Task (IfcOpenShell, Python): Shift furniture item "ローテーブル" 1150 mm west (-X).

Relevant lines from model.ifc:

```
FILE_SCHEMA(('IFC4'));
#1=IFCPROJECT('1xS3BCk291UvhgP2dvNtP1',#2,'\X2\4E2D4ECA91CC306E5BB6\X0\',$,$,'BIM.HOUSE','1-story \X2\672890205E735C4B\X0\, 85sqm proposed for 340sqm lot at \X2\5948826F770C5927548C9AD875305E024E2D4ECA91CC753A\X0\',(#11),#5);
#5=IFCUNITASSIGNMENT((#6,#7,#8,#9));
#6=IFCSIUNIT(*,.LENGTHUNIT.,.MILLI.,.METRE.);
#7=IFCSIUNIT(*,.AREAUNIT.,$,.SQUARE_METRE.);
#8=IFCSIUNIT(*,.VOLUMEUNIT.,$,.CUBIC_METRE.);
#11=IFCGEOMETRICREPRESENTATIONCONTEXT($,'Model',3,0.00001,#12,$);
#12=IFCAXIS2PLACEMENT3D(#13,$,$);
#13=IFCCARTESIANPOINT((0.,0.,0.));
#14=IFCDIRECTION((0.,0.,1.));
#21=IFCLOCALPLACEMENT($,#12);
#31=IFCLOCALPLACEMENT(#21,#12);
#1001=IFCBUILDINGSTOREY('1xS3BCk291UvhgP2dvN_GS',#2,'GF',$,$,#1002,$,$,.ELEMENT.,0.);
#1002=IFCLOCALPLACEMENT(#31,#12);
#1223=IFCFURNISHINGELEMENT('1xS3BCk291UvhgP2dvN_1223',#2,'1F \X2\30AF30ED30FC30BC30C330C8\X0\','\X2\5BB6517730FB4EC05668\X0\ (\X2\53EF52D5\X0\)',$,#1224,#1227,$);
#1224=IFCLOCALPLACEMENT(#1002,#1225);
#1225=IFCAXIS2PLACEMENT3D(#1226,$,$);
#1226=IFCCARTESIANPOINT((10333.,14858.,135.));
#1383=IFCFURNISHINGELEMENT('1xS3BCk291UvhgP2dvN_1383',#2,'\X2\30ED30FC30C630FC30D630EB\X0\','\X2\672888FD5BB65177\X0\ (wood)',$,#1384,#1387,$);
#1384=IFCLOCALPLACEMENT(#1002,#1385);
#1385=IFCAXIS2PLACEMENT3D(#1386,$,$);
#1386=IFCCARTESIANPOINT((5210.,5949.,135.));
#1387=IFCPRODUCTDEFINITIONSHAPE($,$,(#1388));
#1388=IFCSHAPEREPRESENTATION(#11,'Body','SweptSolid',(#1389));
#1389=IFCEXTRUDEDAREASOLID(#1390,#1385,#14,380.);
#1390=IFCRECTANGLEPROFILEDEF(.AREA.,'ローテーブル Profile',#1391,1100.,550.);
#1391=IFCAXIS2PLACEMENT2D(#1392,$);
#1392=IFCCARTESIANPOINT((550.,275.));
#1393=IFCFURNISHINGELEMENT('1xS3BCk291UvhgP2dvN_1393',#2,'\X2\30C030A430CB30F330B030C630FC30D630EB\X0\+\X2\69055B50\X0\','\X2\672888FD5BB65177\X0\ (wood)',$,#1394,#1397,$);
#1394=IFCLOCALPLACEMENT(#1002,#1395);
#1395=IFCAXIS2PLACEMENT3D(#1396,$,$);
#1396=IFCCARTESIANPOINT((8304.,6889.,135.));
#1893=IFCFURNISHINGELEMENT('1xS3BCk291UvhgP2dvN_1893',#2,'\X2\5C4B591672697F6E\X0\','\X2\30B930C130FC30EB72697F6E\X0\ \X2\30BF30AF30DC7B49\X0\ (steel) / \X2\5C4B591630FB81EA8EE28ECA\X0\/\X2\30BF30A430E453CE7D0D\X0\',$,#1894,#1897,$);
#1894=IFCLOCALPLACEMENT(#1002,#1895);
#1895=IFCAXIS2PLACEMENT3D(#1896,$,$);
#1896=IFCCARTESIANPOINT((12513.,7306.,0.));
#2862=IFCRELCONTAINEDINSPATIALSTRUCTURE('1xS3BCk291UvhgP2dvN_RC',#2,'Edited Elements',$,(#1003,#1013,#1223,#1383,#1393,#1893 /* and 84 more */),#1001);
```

```python
import ifcopenshell
import ifcopenshell.api.geometry
import ifcopenshell.util.placement

model = ifcopenshell.open("model.ifc")

item = model.by_guid("1xS3BCk291UvhgP2dvN_1383")
matrix = ifcopenshell.util.placement.get_local_placement(item.ObjectPlacement)
matrix[0, 3] -= 1150.0
ifcopenshell.api.geometry.edit_object_placement(model, product=item, matrix=matrix, is_si=False)

print(ifcopenshell.util.placement.get_local_placement(item.ObjectPlacement).round(3) + 0.0)

model.write("model-out.ifc")
```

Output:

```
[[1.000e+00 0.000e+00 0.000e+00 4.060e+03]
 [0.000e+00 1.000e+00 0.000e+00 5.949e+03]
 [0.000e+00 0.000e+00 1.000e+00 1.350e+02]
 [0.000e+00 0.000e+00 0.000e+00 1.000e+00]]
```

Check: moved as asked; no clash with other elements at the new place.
